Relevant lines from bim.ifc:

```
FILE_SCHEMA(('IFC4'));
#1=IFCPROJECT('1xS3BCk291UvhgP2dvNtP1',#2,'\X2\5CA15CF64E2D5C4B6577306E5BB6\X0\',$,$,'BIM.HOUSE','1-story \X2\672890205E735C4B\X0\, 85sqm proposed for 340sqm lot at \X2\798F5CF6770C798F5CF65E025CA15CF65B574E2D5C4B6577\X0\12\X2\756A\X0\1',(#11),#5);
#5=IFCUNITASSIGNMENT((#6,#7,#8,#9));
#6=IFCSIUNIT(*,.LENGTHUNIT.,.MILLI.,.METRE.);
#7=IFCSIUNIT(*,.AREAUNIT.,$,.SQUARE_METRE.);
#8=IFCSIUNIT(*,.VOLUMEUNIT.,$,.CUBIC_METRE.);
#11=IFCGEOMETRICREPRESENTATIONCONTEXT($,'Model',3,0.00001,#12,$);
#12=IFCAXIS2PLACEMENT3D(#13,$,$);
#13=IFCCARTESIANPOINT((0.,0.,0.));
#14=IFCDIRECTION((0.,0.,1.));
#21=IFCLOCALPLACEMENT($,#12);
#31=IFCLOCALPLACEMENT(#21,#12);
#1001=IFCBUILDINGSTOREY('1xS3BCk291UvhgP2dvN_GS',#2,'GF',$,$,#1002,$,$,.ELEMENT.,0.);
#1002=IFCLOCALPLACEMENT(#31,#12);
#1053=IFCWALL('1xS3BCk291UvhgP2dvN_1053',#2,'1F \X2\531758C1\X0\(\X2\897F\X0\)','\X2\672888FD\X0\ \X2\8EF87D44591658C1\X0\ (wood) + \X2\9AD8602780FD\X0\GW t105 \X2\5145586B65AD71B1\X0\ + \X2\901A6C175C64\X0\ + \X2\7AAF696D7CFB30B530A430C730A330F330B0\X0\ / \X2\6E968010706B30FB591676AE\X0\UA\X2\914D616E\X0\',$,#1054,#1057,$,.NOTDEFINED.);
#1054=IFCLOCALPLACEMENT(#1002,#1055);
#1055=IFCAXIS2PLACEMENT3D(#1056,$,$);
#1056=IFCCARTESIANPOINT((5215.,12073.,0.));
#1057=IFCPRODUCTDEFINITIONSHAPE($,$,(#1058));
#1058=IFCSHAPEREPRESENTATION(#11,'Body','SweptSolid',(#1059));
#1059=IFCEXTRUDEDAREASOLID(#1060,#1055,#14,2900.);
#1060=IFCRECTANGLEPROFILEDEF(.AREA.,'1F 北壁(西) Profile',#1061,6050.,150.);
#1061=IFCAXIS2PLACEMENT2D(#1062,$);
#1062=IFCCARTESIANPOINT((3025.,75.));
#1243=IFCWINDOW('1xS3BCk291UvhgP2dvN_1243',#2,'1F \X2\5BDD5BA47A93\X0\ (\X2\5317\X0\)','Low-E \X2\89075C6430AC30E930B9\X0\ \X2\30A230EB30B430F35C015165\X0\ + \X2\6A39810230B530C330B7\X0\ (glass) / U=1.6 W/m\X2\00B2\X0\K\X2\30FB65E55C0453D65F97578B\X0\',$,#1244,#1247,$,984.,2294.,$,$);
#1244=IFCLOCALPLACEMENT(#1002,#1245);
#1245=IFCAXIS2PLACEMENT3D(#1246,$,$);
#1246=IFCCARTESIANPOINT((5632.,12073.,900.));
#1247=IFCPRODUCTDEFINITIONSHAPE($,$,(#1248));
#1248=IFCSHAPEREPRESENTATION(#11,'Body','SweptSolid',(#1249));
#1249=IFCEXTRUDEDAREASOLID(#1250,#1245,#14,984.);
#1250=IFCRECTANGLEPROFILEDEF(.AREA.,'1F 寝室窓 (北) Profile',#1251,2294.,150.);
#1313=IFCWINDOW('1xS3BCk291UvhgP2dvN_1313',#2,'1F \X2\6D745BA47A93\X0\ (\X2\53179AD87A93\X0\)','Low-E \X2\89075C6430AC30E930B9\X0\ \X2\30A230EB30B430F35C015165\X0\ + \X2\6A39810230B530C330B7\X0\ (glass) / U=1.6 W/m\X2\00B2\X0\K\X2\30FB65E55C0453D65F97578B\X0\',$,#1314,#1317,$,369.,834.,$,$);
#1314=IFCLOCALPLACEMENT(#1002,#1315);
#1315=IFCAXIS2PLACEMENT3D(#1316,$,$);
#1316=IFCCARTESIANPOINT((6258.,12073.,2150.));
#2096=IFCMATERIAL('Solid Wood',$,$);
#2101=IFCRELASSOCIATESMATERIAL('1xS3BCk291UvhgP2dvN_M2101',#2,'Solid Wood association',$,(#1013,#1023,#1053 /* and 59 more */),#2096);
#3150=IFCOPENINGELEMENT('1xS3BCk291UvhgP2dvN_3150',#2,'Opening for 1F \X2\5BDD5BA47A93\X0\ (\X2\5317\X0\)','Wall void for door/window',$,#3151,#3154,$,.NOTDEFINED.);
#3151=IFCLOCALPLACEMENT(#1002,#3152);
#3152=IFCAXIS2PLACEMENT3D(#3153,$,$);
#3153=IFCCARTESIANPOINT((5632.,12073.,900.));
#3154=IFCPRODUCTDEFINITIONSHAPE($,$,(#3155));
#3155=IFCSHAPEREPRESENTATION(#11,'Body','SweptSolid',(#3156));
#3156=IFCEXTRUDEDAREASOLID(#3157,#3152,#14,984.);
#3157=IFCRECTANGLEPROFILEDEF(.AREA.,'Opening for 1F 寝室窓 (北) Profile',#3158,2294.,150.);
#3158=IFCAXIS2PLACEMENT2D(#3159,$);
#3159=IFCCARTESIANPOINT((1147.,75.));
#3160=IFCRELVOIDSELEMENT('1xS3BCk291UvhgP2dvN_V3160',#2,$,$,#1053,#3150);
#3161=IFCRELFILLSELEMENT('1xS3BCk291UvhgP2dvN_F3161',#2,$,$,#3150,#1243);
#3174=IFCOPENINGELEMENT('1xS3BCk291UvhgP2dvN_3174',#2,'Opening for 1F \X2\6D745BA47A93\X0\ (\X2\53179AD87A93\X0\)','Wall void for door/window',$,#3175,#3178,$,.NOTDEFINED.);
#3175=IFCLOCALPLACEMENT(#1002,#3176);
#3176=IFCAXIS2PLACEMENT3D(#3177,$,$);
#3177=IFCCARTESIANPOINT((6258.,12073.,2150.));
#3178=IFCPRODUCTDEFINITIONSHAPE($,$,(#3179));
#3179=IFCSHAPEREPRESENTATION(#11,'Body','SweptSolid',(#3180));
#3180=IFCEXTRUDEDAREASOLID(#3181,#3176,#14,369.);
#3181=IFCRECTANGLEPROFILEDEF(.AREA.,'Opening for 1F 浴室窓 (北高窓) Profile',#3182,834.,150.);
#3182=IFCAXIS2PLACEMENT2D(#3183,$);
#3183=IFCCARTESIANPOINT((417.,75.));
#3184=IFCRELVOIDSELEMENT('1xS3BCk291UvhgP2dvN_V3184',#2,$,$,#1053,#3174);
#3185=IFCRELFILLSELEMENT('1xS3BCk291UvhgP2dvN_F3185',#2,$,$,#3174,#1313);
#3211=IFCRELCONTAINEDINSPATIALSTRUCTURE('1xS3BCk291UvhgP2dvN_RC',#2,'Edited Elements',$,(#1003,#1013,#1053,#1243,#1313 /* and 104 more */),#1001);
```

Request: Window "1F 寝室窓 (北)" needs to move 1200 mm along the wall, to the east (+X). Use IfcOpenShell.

```python
import ifcopenshell
import ifcopenshell.api.geometry
import ifcopenshell.util.placement

model = ifcopenshell.open("bim.ifc")

window = model.by_id(1243)
opening = window.FillsVoids[0].RelatingOpeningElement
wall = opening.VoidsElements[0].RelatingBuildingElement

wall_matrix = ifcopenshell.util.placement.get_local_placement(wall.ObjectPlacement)
shift = wall_matrix[:3, 0] * 1200.0
before = ifcopenshell.util.placement.get_local_placement(window.ObjectPlacement)[:3, 3].copy()

# The window is not placed relative to its opening, so move both.
for product in (opening, window):
    matrix = ifcopenshell.util.placement.get_local_placement(product.ObjectPlacement)
    matrix[:3, 3] += shift
    ifcopenshell.api.geometry.edit_object_placement(model, product=product, matrix=matrix, is_si=False)

after = ifcopenshell.util.placement.get_local_placement(window.ObjectPlacement)[:3, 3]
print("window moved by", (after - before).round(3) + 0.0)

model.write("bim_rev.ifc")
```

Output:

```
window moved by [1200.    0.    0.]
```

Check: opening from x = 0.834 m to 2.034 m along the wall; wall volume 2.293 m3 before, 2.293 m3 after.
